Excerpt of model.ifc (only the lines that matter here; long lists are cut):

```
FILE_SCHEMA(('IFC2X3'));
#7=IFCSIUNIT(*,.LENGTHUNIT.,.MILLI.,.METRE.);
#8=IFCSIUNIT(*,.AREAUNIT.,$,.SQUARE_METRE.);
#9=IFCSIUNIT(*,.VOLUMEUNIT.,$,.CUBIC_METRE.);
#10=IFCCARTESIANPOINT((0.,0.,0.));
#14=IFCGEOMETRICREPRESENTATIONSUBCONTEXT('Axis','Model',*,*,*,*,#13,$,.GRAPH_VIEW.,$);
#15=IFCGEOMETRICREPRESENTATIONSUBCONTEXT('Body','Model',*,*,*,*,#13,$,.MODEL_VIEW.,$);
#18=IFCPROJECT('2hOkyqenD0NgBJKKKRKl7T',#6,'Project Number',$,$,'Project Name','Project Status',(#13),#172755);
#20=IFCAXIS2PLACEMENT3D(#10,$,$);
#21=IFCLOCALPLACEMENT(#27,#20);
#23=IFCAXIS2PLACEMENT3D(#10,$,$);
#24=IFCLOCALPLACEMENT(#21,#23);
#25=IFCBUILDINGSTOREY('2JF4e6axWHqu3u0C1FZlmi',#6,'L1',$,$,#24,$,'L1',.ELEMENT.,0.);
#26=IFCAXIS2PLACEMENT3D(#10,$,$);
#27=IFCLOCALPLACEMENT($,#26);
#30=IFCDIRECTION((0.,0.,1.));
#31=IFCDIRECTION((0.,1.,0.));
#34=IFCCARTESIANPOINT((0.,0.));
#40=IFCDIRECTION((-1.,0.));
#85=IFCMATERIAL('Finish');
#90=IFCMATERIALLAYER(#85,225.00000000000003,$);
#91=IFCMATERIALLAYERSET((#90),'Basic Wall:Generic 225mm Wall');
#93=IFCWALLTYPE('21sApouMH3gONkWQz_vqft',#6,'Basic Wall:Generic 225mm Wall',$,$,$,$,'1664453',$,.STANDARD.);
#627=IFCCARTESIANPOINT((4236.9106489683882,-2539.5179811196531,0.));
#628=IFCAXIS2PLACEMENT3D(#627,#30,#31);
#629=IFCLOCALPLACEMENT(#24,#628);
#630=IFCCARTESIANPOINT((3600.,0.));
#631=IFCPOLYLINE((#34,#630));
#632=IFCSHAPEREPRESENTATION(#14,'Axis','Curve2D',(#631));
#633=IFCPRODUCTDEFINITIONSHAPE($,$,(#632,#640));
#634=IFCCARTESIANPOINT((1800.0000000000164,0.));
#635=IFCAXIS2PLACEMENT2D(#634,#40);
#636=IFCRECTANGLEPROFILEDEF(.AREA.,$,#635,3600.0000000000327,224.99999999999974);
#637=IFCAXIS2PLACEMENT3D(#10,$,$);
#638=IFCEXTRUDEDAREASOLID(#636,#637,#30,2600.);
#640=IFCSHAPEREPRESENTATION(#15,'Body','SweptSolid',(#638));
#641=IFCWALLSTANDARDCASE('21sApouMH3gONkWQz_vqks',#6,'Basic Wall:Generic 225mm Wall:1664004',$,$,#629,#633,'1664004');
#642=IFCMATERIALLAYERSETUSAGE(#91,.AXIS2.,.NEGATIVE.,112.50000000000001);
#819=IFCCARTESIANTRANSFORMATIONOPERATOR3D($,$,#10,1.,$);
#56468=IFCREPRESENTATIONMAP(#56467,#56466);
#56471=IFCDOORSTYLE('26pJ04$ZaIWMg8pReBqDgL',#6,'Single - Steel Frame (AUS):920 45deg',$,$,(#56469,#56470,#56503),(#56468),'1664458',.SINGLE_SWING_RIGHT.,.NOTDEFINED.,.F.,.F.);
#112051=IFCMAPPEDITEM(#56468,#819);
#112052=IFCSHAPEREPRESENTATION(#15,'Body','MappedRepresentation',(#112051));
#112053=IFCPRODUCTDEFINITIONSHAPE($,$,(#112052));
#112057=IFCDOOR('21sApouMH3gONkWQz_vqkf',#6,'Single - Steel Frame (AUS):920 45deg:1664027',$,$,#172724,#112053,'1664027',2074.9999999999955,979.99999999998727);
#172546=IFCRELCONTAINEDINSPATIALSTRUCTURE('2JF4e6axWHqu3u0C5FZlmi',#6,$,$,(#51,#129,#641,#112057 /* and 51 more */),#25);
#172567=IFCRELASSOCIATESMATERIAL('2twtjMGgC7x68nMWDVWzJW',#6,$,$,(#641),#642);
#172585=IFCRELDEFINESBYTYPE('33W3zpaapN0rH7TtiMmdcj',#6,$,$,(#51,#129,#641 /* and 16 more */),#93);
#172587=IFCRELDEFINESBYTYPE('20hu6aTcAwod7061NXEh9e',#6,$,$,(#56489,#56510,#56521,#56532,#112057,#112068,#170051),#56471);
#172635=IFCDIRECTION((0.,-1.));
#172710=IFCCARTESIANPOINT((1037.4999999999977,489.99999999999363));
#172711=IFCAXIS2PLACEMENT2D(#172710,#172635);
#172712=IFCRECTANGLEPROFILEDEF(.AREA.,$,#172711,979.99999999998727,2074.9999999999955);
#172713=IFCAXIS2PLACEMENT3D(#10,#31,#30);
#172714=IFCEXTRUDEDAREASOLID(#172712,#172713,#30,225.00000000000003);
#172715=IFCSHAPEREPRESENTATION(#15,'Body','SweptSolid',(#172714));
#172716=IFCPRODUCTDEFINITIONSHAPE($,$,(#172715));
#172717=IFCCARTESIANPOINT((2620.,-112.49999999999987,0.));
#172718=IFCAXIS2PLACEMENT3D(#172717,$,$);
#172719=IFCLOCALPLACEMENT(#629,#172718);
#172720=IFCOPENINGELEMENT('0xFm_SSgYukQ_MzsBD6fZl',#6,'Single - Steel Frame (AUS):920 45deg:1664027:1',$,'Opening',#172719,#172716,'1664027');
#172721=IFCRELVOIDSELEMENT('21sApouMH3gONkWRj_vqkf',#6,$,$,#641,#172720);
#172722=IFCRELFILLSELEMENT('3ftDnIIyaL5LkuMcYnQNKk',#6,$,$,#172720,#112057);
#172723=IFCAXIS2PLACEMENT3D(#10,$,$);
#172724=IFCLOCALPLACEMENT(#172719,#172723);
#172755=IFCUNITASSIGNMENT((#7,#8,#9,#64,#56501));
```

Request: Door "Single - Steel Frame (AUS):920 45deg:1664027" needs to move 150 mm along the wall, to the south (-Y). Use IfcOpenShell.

```python
import ifcopenshell
import ifcopenshell.api.geometry
import ifcopenshell.util.placement
import ifcopenshell.util.unit

model = ifcopenshell.open("model.ifc")
unit_scale = ifcopenshell.util.unit.calculate_unit_scale(model)

door = model.by_guid("21sApouMH3gONkWQz_vqkf")
opening = door.FillsVoids[0].RelatingOpeningElement
wall = opening.VoidsElements[0].RelatingBuildingElement

wall_matrix = ifcopenshell.util.placement.get_local_placement(wall.ObjectPlacement)
shift = wall_matrix[:3, 0] * -0.15 / unit_scale
before = ifcopenshell.util.placement.get_local_placement(door.ObjectPlacement)[:3, 3].copy()

# The door is placed relative to its opening, so it follows when the opening moves.
matrix = ifcopenshell.util.placement.get_local_placement(opening.ObjectPlacement)
matrix[:3, 3] += shift
ifcopenshell.api.geometry.edit_object_placement(
    model, product=opening, matrix=matrix, is_si=False, should_transform_children=True
)

after = ifcopenshell.util.placement.get_local_placement(door.ObjectPlacement)[:3, 3]
print("door moved by", (after - before).round(3) + 0.0)

model.write("model_v2.ifc")
```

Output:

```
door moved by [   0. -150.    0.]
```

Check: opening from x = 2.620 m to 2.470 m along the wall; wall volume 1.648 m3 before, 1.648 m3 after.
